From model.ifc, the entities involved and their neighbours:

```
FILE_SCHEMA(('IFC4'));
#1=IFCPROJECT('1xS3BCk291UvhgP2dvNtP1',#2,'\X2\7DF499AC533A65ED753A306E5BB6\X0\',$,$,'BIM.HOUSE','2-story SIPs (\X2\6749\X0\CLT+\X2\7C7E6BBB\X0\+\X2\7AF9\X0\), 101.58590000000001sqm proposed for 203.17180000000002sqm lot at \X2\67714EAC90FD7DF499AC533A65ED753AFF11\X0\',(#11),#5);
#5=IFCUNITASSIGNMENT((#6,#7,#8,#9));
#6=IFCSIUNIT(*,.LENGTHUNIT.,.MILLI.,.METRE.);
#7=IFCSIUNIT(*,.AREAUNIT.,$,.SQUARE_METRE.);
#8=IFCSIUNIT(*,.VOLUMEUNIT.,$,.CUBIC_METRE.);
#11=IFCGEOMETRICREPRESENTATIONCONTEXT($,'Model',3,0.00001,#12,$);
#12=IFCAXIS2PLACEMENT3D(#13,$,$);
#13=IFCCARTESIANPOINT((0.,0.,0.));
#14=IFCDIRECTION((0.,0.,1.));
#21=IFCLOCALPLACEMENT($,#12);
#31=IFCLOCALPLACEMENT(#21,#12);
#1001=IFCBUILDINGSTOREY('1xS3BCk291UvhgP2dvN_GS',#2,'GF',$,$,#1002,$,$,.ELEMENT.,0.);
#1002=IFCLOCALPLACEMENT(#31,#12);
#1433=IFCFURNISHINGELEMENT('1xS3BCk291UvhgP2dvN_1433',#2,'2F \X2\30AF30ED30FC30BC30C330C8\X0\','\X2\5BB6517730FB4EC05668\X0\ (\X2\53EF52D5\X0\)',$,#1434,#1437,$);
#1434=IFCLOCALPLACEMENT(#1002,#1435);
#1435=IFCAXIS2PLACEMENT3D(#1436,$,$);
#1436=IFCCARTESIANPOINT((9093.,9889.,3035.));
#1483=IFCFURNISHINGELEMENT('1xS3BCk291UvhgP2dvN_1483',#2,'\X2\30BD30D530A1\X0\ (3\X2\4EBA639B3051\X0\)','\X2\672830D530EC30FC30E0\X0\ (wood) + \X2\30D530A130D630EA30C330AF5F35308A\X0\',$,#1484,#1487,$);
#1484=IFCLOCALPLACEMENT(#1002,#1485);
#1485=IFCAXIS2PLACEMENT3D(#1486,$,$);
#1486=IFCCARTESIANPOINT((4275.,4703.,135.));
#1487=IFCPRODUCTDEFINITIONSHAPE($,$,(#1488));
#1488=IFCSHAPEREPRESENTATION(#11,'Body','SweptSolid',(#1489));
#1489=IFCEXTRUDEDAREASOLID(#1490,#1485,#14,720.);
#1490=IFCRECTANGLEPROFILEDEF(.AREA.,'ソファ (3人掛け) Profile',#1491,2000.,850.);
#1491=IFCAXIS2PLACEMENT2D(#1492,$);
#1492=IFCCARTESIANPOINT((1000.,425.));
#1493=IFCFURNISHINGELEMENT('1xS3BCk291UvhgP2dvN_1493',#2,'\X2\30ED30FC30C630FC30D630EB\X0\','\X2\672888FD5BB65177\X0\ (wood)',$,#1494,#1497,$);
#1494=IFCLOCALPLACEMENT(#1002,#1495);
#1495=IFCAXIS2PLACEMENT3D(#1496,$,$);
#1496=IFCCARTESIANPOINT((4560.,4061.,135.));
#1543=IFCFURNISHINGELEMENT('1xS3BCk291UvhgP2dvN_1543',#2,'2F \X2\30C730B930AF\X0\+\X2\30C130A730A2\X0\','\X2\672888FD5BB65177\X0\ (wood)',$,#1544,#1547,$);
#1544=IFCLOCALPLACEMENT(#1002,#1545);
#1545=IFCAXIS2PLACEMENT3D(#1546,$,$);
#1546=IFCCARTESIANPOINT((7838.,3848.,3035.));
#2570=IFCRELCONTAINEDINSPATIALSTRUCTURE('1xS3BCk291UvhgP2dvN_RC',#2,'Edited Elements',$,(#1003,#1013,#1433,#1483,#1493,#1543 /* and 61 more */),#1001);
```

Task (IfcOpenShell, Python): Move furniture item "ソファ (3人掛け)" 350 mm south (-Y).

```python
import ifcopenshell
import ifcopenshell.api.geometry
import ifcopenshell.util.placement

model = ifcopenshell.open("model.ifc")

item = model.by_guid("1xS3BCk291UvhgP2dvN_1483")
matrix = ifcopenshell.util.placement.get_local_placement(item.ObjectPlacement)
matrix[1, 3] -= 350.0
ifcopenshell.api.geometry.edit_object_placement(model, product=item, matrix=matrix, is_si=False)

print(ifcopenshell.util.placement.get_local_placement(item.ObjectPlacement).round(3) + 0.0)

model.write("model-out.ifc")
```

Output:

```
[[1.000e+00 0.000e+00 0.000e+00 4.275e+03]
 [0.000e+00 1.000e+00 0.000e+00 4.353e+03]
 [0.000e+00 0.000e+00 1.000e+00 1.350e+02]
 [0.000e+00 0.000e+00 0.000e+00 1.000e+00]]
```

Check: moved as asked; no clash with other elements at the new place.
